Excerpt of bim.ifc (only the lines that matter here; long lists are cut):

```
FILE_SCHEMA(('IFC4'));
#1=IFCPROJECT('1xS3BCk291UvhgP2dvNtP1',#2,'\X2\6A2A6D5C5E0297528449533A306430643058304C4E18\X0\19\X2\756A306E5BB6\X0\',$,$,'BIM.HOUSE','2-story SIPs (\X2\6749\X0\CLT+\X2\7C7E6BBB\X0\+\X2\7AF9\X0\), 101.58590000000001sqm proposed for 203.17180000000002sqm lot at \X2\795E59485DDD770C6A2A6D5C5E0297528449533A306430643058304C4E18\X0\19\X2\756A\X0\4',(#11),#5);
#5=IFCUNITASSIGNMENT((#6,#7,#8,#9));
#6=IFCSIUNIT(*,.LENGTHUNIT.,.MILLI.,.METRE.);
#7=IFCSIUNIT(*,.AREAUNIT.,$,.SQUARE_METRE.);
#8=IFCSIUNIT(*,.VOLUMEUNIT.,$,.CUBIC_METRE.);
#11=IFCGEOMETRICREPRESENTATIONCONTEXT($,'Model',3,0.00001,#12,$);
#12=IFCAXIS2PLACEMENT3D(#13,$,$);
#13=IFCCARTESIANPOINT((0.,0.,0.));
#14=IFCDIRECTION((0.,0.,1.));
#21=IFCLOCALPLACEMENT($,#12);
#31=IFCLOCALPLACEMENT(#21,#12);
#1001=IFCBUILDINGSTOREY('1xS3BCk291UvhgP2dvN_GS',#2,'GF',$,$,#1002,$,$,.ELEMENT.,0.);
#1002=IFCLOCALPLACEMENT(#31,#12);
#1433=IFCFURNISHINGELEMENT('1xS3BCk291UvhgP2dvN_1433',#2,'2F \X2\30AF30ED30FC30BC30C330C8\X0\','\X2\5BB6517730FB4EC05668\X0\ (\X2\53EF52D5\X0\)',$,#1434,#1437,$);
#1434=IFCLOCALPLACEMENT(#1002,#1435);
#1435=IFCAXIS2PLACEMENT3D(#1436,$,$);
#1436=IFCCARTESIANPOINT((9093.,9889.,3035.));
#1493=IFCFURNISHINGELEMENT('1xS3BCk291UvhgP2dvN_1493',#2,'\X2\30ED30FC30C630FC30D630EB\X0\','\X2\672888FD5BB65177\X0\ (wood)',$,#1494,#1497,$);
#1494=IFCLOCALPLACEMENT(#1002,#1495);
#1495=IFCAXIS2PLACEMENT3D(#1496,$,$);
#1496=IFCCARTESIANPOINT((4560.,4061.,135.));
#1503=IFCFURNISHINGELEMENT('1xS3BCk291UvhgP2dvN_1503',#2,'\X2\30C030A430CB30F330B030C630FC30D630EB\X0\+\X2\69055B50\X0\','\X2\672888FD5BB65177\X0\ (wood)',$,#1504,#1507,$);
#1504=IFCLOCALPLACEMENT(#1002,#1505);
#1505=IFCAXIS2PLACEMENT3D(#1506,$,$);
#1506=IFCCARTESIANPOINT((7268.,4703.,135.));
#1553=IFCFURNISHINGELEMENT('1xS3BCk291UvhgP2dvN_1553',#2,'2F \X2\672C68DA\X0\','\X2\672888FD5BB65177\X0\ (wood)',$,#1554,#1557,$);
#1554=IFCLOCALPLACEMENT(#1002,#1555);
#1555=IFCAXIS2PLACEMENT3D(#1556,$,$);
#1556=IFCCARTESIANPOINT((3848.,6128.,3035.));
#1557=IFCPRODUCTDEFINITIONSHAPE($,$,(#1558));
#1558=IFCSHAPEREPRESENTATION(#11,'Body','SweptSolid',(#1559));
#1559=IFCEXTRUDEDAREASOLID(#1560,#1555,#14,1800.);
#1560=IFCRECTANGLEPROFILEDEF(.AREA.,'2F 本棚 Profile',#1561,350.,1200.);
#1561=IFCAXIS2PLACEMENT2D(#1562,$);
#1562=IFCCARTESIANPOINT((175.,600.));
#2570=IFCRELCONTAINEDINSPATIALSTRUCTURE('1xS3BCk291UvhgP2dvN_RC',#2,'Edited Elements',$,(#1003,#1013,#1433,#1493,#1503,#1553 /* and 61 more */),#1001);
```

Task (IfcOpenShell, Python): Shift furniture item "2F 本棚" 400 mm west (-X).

```python
import ifcopenshell
import ifcopenshell.api.geometry
import ifcopenshell.util.placement
import ifcopenshell.util.unit

model = ifcopenshell.open("bim.ifc")
unit_scale = ifcopenshell.util.unit.calculate_unit_scale(model)

item = model.by_id(1553)
matrix = ifcopenshell.util.placement.get_local_placement(item.ObjectPlacement)
matrix[0, 3] -= 0.4 / unit_scale
ifcopenshell.api.geometry.edit_object_placement(model, product=item, matrix=matrix, is_si=False)

print(ifcopenshell.util.placement.get_local_placement(item.ObjectPlacement).round(3) + 0.0)

model.write("bim_edited.ifc")
```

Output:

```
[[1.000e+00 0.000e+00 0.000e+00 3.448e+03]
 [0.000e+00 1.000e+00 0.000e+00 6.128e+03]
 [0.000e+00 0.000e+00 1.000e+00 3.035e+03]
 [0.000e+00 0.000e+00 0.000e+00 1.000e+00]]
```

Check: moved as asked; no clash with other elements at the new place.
